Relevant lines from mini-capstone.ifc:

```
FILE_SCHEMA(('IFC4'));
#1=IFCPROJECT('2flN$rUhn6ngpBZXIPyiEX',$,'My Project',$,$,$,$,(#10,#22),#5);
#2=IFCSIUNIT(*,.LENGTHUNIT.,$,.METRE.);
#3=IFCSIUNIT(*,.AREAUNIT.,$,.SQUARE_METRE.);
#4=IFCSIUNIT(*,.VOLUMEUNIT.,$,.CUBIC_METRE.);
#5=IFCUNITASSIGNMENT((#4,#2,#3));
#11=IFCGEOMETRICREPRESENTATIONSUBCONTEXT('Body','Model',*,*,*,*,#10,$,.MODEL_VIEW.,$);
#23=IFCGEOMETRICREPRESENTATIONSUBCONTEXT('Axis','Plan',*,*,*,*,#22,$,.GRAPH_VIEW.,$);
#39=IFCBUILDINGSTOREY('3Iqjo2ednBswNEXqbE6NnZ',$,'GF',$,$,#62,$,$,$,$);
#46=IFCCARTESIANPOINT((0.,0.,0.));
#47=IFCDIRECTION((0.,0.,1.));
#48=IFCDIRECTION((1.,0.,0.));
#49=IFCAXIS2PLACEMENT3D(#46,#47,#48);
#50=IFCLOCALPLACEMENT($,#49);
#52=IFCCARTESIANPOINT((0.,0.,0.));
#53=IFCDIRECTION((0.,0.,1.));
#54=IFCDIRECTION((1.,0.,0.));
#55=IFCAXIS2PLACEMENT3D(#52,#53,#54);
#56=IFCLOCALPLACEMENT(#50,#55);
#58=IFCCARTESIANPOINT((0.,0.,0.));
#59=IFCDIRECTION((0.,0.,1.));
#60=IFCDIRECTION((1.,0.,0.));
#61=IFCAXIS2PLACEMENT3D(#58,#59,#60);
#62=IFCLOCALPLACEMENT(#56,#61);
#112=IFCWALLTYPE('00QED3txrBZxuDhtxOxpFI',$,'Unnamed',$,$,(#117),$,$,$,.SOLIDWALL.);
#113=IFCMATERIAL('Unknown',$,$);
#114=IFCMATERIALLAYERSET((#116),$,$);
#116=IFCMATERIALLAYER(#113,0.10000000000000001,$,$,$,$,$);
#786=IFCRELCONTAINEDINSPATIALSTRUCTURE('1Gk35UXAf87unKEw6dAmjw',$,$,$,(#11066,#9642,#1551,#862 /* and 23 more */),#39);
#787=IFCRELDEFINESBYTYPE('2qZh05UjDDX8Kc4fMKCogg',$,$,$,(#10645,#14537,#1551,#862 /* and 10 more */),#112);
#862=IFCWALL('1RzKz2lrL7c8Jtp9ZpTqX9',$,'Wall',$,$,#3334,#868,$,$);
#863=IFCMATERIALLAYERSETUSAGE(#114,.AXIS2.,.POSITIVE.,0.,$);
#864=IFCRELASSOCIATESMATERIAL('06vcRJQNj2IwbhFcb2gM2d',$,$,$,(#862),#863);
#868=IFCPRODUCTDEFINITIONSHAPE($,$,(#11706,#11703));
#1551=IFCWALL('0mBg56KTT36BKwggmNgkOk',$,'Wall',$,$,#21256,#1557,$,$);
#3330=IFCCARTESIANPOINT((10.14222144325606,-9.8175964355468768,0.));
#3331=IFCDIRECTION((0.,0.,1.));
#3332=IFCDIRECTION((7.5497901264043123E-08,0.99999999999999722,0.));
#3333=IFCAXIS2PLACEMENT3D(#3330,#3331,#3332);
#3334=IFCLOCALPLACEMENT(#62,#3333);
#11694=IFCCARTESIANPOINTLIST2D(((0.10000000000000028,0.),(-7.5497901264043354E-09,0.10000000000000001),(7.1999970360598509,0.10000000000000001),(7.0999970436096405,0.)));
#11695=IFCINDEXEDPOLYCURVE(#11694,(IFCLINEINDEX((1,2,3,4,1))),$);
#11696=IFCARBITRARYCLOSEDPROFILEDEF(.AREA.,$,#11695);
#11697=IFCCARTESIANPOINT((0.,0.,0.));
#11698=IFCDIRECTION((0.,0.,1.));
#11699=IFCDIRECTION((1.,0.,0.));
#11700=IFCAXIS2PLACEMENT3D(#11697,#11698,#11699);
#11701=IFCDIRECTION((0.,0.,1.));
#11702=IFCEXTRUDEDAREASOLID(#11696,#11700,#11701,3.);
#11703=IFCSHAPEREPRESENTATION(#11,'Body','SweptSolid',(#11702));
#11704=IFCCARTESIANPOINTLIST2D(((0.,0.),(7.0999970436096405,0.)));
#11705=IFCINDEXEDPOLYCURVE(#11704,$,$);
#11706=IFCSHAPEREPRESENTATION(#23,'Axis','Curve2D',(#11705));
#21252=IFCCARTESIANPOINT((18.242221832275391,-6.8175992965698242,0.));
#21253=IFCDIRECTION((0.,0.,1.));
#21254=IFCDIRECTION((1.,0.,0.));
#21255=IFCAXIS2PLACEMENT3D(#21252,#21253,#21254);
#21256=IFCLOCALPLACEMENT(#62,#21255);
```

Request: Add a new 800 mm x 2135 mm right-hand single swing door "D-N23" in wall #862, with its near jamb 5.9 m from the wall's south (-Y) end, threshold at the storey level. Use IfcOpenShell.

```python
import numpy as np
import ifcopenshell
import ifcopenshell.api.feature
import ifcopenshell.api.geometry
import ifcopenshell.api.root
import ifcopenshell.api.spatial
import ifcopenshell.geom
import ifcopenshell.util.element
import ifcopenshell.util.placement
import ifcopenshell.util.representation
import ifcopenshell.util.shape
import ifcopenshell.util.unit

model = ifcopenshell.open("mini-capstone.ifc")
unit_scale = ifcopenshell.util.unit.calculate_unit_scale(model)
settings = ifcopenshell.geom.settings()


def volume(element):
    """Net volume in cubic metres, openings subtracted."""
    shape = ifcopenshell.geom.create_shape(settings, element)
    return ifcopenshell.util.shape.get_volume(shape.geometry)


wall = model.by_guid("1RzKz2lrL7c8Jtp9ZpTqX9")
storey = ifcopenshell.util.element.get_container(wall, ifc_class="IfcBuildingStorey")
context = ifcopenshell.util.representation.get_context(model, "Model", "Body", "MODEL_VIEW")
before = volume(wall)

width, height, from_end, sill = 0.8, 2.135, 5.9, 0.0  # metres

# The wall runs along its own X axis, and the end named is its -X end.
wall_shape = ifcopenshell.geom.create_shape(settings, wall)
x, y, z = ifcopenshell.util.shape.get_vertices(wall_shape.geometry).T
start = x.min() + from_end
face, thickness = float(y.min()), float(y.max() - y.min())
wall_matrix = ifcopenshell.util.placement.get_local_placement(wall.ObjectPlacement)
level = ifcopenshell.util.placement.get_local_placement(storey.ObjectPlacement)[2, 3]


def in_wall(x, y):
    """Placement at x, y metres in the wall's axes, at sill height."""
    matrix = wall_matrix.copy()
    matrix[:, 3] = wall_matrix @ np.array([x / unit_scale, y / unit_scale, 0.0, 1.0])
    matrix[2, 3] = level + sill / unit_scale
    return matrix


# Opening: a box that overshoots both wall faces by 50 mm.
opening = ifcopenshell.api.root.create_entity(model, ifc_class="IfcOpeningElement", predefined_type="OPENING")
box = ifcopenshell.api.geometry.add_wall_representation(
    model, context=context, length=width, height=height, thickness=thickness + 0.1
)
ifcopenshell.api.geometry.assign_representation(model, product=opening, representation=box)
ifcopenshell.api.geometry.edit_object_placement(model, product=opening, matrix=in_wall(start, face - 0.05), is_si=False)
ifcopenshell.api.feature.add_feature(model, feature=opening, element=wall)

door = ifcopenshell.api.root.create_entity(model, ifc_class="IfcDoor", name="D-N23", predefined_type="DOOR")
door.OverallWidth, door.OverallHeight = width / unit_scale, height / unit_scale
door.OperationType = "SINGLE_SWING_RIGHT"
body = ifcopenshell.api.geometry.add_door_representation(
    model,
    context=context,
    overall_width=door.OverallWidth,
    overall_height=door.OverallHeight,
    operation_type="SINGLE_SWING_RIGHT",
    lining_properties={"LiningDepth": thickness / unit_scale, "ThresholdDepth": thickness / unit_scale},
)
ifcopenshell.api.geometry.assign_representation(model, product=door, representation=body)
ifcopenshell.api.spatial.assign_container(model, products=[door], relating_structure=storey)
ifcopenshell.api.feature.add_filling(model, opening=opening, element=door)

# The lining spans the wall, so the door starts at the wall face.
ifcopenshell.api.geometry.edit_object_placement(model, product=door, matrix=in_wall(start, face), is_si=False)

after = volume(wall)

print(f"wall volume {before:.3f} -> {after:.3f} m3")

model.write("mini-capstone_edited.ifc")
```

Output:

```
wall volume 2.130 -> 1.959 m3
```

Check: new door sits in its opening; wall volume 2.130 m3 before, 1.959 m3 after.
